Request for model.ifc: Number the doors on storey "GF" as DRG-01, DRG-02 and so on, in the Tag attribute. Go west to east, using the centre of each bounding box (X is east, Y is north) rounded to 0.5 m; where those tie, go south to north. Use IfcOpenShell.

First a look at what the model holds.

```python
import ifcopenshell
import ifcopenshell.util.element
import ifcopenshell.util.placement

model = ifcopenshell.open("model.ifc")
print(model.schema)
storey = next(s for s in model.by_type("IfcBuildingStorey") if s.Name == "GF")
doors = [e for e in ifcopenshell.util.element.get_decomposition(storey) if e.is_a("IfcDoor")]
for e in sorted(doors, key=lambda e: e.id()):
    origin = ifcopenshell.util.placement.get_local_placement(e.ObjectPlacement)[:3, 3]
    print(e.id(), e.Tag, e.Name, origin.round(2) + 0.0, sep=" | ")
```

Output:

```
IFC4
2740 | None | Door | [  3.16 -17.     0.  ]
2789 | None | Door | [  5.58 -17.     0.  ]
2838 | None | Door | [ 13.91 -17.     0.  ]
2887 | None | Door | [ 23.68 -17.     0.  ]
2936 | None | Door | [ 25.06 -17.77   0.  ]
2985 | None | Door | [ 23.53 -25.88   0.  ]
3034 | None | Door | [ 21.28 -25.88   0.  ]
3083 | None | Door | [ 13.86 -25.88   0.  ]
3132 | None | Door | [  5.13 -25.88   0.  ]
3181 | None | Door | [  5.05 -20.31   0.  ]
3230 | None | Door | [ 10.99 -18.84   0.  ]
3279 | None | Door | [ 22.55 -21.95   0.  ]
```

```python
import ifcopenshell
import ifcopenshell.geom
import ifcopenshell.util.element
import ifcopenshell.util.shape

model = ifcopenshell.open("model.ifc")
settings = ifcopenshell.geom.settings()
settings.set("use-world-coords", True)


def centre(element):
    shape = ifcopenshell.geom.create_shape(settings, element)
    return ifcopenshell.util.shape.get_bbox_centroid(shape.geometry)


storey = next(s for s in model.by_type("IfcBuildingStorey") if s.Name == "GF")
doors = [e for e in ifcopenshell.util.element.get_decomposition(storey) if e.is_a("IfcDoor")]

# Insertion points can sit at a corner or the storey origin, so sort by the geometry (in metres).
centres = {e: centre(e) for e in doors}
doors.sort(key=lambda e: (round(centres[e][0] / 0.5), centres[e][1]))

for i, e in enumerate(doors, start=1):
    number = f"DRG-{i:02d}"
    e.Tag = number
    print(e.id(), number)

model.write("model_edited.ifc")
```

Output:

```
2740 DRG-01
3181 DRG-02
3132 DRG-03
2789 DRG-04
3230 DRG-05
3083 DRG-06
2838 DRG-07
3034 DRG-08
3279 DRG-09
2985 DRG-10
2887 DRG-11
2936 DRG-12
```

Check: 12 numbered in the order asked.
